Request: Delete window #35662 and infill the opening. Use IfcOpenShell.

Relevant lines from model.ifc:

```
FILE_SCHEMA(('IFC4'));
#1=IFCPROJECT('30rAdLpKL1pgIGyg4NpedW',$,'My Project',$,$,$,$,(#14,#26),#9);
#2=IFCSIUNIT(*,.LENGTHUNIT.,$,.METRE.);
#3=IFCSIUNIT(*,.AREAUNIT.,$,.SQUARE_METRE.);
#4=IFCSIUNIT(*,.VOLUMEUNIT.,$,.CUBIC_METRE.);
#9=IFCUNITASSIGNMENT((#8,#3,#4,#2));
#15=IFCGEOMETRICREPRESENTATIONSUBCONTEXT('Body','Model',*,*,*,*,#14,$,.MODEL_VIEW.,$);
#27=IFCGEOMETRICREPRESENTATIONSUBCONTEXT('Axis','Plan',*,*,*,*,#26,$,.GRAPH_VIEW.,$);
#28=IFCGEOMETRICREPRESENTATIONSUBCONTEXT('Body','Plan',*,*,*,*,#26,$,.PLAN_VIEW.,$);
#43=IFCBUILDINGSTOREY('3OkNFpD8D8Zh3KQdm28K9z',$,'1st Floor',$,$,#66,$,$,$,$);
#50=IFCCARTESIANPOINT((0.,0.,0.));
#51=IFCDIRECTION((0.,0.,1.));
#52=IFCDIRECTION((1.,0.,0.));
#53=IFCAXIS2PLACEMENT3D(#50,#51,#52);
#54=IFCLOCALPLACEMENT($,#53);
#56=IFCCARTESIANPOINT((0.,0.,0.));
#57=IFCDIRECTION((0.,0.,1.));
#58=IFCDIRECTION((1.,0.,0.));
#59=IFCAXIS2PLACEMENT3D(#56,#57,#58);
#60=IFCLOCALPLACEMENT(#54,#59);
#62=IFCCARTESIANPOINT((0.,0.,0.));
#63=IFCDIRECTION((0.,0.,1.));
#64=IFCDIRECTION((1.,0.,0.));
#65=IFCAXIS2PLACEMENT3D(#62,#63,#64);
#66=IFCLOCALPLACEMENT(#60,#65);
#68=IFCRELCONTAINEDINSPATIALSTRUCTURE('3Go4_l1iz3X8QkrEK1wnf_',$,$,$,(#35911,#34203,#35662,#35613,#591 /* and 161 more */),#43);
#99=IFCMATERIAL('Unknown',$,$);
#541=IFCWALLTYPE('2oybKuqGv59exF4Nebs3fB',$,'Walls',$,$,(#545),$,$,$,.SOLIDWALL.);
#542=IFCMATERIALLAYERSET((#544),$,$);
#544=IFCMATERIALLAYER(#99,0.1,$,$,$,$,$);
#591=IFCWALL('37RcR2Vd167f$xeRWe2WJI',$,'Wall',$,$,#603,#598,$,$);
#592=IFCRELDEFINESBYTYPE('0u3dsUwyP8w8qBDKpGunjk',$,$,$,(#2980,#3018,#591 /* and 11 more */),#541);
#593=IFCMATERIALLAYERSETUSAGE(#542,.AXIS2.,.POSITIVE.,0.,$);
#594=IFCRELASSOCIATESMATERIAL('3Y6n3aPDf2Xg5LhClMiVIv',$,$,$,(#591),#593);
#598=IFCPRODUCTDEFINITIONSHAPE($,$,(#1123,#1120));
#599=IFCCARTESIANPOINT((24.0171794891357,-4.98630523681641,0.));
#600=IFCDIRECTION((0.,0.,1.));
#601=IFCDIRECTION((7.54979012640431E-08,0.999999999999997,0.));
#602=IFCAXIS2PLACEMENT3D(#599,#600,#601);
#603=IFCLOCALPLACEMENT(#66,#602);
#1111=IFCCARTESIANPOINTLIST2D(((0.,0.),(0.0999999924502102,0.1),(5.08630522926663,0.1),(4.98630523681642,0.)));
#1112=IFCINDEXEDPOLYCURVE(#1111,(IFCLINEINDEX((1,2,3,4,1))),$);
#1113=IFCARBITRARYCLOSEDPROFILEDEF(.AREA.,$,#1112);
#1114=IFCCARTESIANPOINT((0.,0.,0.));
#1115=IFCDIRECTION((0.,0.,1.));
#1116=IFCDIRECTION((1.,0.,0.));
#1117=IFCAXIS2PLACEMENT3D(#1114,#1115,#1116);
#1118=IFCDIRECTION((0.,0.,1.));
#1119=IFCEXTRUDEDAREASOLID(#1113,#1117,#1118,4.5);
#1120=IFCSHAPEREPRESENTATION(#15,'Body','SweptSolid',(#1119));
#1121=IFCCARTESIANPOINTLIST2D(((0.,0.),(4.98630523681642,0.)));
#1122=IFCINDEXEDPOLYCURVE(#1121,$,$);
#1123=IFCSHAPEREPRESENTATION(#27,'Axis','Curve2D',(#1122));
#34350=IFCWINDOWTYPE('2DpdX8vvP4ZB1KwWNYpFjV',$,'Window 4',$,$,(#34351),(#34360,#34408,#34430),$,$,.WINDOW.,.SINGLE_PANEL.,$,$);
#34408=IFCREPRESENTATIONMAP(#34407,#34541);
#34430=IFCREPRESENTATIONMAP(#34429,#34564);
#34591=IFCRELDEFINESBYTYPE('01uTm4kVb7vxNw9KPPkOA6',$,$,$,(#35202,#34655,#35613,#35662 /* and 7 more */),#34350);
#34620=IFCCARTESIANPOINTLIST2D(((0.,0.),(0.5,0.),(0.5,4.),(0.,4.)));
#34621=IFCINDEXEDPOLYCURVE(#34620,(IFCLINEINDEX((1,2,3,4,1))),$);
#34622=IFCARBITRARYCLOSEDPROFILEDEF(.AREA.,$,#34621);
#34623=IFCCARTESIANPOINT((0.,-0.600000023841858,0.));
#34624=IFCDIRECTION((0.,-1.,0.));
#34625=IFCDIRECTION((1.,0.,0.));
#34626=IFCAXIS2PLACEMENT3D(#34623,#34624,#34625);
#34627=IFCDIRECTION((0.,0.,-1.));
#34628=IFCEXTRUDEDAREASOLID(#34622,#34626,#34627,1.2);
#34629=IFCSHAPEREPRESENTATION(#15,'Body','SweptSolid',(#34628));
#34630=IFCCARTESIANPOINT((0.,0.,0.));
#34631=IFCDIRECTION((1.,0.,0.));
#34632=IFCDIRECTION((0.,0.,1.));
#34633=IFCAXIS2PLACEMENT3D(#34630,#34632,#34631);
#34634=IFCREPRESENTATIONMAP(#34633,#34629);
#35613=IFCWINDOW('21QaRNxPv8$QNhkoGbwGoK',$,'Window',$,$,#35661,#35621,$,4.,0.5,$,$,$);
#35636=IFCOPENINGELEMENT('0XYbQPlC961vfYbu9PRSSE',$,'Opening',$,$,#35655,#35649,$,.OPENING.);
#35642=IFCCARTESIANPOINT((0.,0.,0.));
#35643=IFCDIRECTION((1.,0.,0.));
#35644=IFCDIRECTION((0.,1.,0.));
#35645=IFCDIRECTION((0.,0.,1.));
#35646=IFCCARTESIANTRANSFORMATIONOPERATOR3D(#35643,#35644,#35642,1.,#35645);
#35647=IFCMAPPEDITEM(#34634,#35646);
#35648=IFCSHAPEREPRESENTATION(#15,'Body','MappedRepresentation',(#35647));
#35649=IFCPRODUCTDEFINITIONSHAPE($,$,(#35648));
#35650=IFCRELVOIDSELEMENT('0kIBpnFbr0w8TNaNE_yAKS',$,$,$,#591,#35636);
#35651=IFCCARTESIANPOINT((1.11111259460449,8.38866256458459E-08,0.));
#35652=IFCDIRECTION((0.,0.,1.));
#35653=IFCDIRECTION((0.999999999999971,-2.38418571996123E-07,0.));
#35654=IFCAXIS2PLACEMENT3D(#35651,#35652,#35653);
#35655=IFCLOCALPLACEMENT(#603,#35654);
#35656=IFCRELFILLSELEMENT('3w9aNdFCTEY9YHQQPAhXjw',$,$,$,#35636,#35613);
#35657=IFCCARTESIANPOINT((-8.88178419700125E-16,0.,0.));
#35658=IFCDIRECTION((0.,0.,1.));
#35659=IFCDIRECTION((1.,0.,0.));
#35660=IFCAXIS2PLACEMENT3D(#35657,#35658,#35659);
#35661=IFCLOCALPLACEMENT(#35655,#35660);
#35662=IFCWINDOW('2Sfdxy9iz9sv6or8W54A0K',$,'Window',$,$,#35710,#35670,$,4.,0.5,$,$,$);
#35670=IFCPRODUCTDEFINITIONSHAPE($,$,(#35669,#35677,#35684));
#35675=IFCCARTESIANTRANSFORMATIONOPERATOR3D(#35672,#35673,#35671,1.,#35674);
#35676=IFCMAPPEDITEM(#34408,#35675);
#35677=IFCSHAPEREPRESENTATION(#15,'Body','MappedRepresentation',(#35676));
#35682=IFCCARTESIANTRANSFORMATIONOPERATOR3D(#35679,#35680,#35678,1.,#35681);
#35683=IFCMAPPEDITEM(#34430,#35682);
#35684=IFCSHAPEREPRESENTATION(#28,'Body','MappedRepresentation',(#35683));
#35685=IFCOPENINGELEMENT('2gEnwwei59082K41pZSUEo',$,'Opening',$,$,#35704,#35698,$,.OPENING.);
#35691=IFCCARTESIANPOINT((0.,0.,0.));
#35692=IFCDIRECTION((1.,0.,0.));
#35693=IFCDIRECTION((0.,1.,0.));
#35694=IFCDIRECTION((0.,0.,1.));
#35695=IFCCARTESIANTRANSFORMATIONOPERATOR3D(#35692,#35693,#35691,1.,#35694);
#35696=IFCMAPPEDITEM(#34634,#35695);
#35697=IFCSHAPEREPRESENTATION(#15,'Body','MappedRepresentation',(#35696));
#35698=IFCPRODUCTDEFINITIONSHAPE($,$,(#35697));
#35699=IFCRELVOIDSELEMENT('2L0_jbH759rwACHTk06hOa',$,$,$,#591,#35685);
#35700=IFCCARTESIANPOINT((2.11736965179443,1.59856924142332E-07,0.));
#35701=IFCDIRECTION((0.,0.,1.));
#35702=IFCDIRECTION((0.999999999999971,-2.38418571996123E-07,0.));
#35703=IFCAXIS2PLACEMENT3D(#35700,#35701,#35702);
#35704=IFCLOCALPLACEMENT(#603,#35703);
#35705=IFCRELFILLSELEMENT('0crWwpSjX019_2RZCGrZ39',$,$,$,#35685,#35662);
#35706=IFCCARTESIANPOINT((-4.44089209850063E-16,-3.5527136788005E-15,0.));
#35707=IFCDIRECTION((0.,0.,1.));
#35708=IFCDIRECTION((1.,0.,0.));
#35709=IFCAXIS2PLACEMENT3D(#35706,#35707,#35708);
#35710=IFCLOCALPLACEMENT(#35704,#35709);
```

```python
import ifcopenshell
import ifcopenshell.api.feature
import ifcopenshell.api.root
import ifcopenshell.geom
import ifcopenshell.util.shape

model = ifcopenshell.open("model.ifc")
settings = ifcopenshell.geom.settings()


def volume(element):
    """Net volume in cubic metres, openings subtracted."""
    shape = ifcopenshell.geom.create_shape(settings, element)
    return ifcopenshell.util.shape.get_volume(shape.geometry)


window = model.by_id(35662)
opening = window.FillsVoids[0].RelatingOpeningElement
wall = opening.VoidsElements[0].RelatingBuildingElement
before = volume(wall)

ifcopenshell.api.root.remove_product(model, product=window)
ifcopenshell.api.feature.remove_feature(model, feature=opening)

after = volume(wall)

print(f"wall volume {before:.3f} -> {after:.3f} m3")

model.write("model_rev.ifc")
```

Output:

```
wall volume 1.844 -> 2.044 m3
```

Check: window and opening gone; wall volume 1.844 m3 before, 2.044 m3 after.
